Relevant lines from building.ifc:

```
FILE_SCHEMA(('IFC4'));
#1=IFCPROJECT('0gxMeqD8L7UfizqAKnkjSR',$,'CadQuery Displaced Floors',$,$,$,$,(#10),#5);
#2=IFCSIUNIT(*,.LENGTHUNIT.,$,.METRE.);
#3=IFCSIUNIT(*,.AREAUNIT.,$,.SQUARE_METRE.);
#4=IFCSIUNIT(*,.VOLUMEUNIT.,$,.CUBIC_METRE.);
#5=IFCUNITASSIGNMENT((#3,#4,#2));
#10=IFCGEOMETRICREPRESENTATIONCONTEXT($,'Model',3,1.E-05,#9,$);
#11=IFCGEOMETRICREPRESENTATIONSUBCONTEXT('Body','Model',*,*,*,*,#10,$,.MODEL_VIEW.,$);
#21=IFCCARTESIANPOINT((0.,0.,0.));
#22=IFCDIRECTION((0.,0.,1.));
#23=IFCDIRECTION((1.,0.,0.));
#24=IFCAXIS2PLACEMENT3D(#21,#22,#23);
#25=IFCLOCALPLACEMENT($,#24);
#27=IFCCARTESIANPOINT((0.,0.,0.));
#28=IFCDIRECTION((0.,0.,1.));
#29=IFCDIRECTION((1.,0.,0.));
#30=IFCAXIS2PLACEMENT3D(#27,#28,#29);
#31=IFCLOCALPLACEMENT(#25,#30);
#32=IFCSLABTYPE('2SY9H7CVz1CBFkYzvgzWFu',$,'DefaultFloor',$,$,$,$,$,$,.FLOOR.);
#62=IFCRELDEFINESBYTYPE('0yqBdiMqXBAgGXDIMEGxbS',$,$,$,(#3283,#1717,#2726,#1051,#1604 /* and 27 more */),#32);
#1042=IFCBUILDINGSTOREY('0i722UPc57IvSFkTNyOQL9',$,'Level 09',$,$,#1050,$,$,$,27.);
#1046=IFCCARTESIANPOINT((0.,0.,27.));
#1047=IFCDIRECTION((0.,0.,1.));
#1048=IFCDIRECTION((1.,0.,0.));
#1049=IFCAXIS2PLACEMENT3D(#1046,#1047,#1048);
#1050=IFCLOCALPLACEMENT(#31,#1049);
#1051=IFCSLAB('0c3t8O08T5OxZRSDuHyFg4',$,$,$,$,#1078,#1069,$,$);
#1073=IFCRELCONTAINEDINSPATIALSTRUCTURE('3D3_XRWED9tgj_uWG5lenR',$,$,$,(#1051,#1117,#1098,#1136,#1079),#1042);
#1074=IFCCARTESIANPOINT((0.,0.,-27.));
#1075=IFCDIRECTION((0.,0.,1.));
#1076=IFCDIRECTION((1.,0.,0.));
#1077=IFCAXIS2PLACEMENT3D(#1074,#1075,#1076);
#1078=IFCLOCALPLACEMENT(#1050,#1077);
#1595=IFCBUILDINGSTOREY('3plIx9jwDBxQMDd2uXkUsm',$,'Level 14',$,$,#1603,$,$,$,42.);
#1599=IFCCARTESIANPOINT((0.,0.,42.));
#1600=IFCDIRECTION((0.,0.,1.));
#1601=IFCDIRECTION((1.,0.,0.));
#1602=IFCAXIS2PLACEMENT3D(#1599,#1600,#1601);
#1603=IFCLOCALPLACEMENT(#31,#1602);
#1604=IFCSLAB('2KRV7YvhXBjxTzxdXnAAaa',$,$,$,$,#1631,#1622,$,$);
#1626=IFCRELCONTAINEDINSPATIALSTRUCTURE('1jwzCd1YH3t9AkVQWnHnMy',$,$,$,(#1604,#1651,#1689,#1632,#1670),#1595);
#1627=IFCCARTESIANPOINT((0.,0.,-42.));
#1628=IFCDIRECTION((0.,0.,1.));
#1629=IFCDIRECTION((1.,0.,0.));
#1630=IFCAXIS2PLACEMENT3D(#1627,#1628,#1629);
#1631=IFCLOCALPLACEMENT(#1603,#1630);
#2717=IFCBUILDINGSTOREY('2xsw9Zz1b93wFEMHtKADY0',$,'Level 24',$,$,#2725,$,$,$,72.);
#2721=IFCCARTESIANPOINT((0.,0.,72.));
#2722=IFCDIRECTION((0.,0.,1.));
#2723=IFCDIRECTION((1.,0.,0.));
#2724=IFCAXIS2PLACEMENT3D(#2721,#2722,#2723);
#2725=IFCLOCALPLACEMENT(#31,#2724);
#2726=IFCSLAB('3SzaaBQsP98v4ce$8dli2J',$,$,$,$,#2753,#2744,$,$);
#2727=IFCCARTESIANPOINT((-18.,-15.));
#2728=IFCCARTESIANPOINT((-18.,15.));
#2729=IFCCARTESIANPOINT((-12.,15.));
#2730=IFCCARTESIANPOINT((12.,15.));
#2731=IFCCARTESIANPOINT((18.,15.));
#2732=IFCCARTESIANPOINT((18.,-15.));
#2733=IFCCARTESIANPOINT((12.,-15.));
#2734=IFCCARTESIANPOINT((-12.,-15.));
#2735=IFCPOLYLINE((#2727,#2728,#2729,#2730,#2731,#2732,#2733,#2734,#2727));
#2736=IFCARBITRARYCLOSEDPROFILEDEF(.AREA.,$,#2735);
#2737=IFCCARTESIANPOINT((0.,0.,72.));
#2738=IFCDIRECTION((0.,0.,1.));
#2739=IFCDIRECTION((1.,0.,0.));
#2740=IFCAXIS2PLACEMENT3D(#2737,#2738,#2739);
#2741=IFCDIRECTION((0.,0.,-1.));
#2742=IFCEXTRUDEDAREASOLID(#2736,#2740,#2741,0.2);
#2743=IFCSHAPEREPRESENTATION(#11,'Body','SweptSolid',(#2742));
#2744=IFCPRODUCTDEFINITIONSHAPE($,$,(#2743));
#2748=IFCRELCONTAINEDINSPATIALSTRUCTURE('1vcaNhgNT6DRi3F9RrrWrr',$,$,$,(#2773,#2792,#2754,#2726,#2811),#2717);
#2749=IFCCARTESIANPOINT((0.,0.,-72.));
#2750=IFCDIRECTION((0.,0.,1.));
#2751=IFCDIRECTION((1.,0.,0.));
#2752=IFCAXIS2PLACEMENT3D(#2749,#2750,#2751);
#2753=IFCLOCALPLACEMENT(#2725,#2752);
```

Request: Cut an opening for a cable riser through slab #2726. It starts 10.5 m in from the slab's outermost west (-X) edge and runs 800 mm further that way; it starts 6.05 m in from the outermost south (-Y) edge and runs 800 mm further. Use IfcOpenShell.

```python
import numpy as np
import ifcopenshell
import ifcopenshell.api.feature
import ifcopenshell.api.geometry
import ifcopenshell.api.root
import ifcopenshell.geom
import ifcopenshell.util.placement
import ifcopenshell.util.representation
import ifcopenshell.util.shape
import ifcopenshell.util.unit

model = ifcopenshell.open("building.ifc")
unit_scale = ifcopenshell.util.unit.calculate_unit_scale(model)
settings = ifcopenshell.geom.settings()


def volume(element):
    """Net volume in cubic metres, openings subtracted."""
    shape = ifcopenshell.geom.create_shape(settings, element)
    return ifcopenshell.util.shape.get_volume(shape.geometry)


slab = model.by_guid("3SzaaBQsP98v4ce$8dli2J")
before = volume(slab)

# Extent in the slab's own axes, in metres. The edges named are its -X and -Y sides.
slab_shape = ifcopenshell.geom.create_shape(settings, slab)
vertices = ifcopenshell.util.shape.get_vertices(slab_shape.geometry)
x_min, y_min, bottom = vertices.min(axis=0)
top = vertices[:, 2].max()

opening = ifcopenshell.api.root.create_entity(model, ifc_class="IfcOpeningElement", name="Cable riser opening", predefined_type="OPENING")
context = ifcopenshell.util.representation.get_context(model, "Model", "Body", "MODEL_VIEW")
width, depth = 0.8, 0.8
outline = [(0.0, 0.0), (width, 0.0), (width, depth), (0.0, depth), (0.0, 0.0)]
# Overshoot both faces by 50 mm so the cut is clean.
shape = ifcopenshell.api.geometry.add_slab_representation(
    model, context=context, depth=top - bottom + 0.1, polyline=outline
)
ifcopenshell.api.geometry.assign_representation(model, product=opening, representation=shape)

matrix = ifcopenshell.util.placement.get_local_placement(slab.ObjectPlacement)
matrix[:, 3] = matrix @ np.append(np.array([x_min + 10.5, y_min + 6.05, bottom - 0.05]) / unit_scale, 1.0)
ifcopenshell.api.geometry.edit_object_placement(model, product=opening, matrix=matrix, is_si=False)
ifcopenshell.api.feature.add_feature(model, feature=opening, element=slab)

after = volume(slab)

print(f"slab volume {before:.3f} -> {after:.3f} m3")

model.write("building_v2.ifc")
```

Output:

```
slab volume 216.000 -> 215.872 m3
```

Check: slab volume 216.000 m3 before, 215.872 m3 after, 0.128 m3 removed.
